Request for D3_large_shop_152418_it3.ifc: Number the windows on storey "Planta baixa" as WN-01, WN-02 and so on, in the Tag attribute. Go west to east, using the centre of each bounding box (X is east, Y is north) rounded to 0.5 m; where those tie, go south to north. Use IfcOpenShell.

First a look at what the model holds.

```python
import ifcopenshell
import ifcopenshell.util.element
import ifcopenshell.util.placement

model = ifcopenshell.open("D3_large_shop_152418_it3.ifc")
print(model.schema)
storey = next(s for s in model.by_type("IfcBuildingStorey") if s.Name == "Planta baixa")
windows = [e for e in ifcopenshell.util.element.get_decomposition(storey) if e.is_a("IfcWindow")]
for e in sorted(windows, key=lambda e: e.id()):
    origin = ifcopenshell.util.placement.get_local_placement(e.ObjectPlacement)[:3, 3]
    print(e.id(), e.Tag, e.Name, origin.round(2) + 0.0, sep=" | ")
```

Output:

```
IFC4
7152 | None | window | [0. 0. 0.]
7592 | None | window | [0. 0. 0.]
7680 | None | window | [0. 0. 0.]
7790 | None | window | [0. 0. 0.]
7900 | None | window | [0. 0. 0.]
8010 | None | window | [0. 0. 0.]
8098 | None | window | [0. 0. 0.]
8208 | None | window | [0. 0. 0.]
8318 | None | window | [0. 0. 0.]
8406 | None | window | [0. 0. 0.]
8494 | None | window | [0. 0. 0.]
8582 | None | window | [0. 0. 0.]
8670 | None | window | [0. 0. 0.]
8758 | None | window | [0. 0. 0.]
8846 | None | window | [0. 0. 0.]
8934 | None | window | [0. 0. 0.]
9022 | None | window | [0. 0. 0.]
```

```python
import ifcopenshell
import ifcopenshell.geom
import ifcopenshell.util.element
import ifcopenshell.util.shape

model = ifcopenshell.open("D3_large_shop_152418_it3.ifc")
settings = ifcopenshell.geom.settings()
settings.set("use-world-coords", True)


def centre(element):
    shape = ifcopenshell.geom.create_shape(settings, element)
    return ifcopenshell.util.shape.get_bbox_centroid(shape.geometry)


storey = next(s for s in model.by_type("IfcBuildingStorey") if s.Name == "Planta baixa")
windows = [e for e in ifcopenshell.util.element.get_decomposition(storey) if e.is_a("IfcWindow")]

# Insertion points can sit at a corner or the storey origin, so sort by the geometry (in metres).
centres = {e: centre(e) for e in windows}
windows.sort(key=lambda e: (round(centres[e][0] / 0.5), centres[e][1]))

for i, e in enumerate(windows, start=1):
    number = f"WN-{i:02d}"
    e.Tag = number
    print(e.id(), number)

model.write("D3_large_shop_152418_it3_edited.ifc")
```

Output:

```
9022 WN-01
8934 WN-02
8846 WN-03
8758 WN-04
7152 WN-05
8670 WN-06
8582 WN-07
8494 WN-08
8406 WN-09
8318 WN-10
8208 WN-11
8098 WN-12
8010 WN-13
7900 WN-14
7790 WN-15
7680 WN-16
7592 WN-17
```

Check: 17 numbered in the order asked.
